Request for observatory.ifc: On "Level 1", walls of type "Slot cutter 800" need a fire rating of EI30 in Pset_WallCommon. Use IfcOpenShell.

First a look at what the model holds.

```python
import ifcopenshell
import ifcopenshell.util.element

model = ifcopenshell.open("observatory.ifc")
print(model.schema)
storey = next(s for s in model.by_type("IfcBuildingStorey") if s.Name == "Level 1")
walls = [e for e in ifcopenshell.util.element.get_decomposition(storey) if e.is_a("IfcWall")]
seen = {}
for e in walls:
    element_type = ifcopenshell.util.element.get_type(e)
    key = (element_type.Name if element_type != e and element_type else None, ifcopenshell.util.element.get_pset(e, "Pset_WallCommon", "FireRating"))
    seen[key] = seen.get(key, 0) + 1
for (name, value), count in sorted(seen.items(), key=str):
    print(count, "x", name, "|", value)
```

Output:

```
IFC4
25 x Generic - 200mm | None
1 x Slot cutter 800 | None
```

```python
import ifcopenshell
import ifcopenshell.api.pset
import ifcopenshell.util.element

model = ifcopenshell.open("observatory.ifc")

storey = next(s for s in model.by_type("IfcBuildingStorey") if s.Name == "Level 1")
walls = [e for e in ifcopenshell.util.element.get_decomposition(storey) if e.is_a("IfcWall")]

count = 0
for e in walls:
    element_type = ifcopenshell.util.element.get_type(e)
    if element_type in (None, e) or element_type.Name != "Slot cutter 800":
        continue
    # add_pset returns the element's existing set when there is one.
    pset = ifcopenshell.api.pset.add_pset(model, product=e, name="Pset_WallCommon")
    ifcopenshell.api.pset.edit_pset(model, pset=pset, properties={"FireRating": "EI30"})
    count += 1

print(count, "walls updated")

model.write("observatory-out.ifc")
```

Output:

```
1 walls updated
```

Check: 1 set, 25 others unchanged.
